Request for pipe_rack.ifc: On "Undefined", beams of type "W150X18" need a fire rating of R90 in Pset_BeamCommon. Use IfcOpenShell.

First a look at what the model holds.

```python
import ifcopenshell
import ifcopenshell.util.element

model = ifcopenshell.open("pipe_rack.ifc")
print(model.schema)
storey = next(s for s in model.by_type("IfcBuildingStorey") if s.Name == "Undefined")
beams = [e for e in ifcopenshell.util.element.get_decomposition(storey) if e.is_a("IfcBeam")]
seen = {}
for e in beams:
    element_type = ifcopenshell.util.element.get_type(e)
    key = (element_type.Name if element_type != e and element_type else None, ifcopenshell.util.element.get_pset(e, "Pset_BeamCommon", "FireRating"))
    seen[key] = seen.get(key, 0) + 1
for (name, value), count in sorted(seen.items(), key=str):
    print(count, "x", name, "|", value)
```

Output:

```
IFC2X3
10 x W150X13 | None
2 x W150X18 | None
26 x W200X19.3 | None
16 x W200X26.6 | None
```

```python
import ifcopenshell
import ifcopenshell.api.pset
import ifcopenshell.util.element

model = ifcopenshell.open("pipe_rack.ifc")

storey = next(s for s in model.by_type("IfcBuildingStorey") if s.Name == "Undefined")
beams = [e for e in ifcopenshell.util.element.get_decomposition(storey) if e.is_a("IfcBeam")]

count = 0
for e in beams:
    element_type = ifcopenshell.util.element.get_type(e)
    if element_type in (None, e) or element_type.Name != "W150X18":
        continue
    found = ifcopenshell.util.element.get_pset(e, "Pset_BeamCommon", should_inherit=False)
    if found:
        pset = model.by_id(found["id"])
        if len(ifcopenshell.util.element.get_elements_by_pset(pset)) > 1:
            pset = ifcopenshell.api.pset.unshare_pset(model, products=[e], pset=pset)[0]
    else:
        pset = ifcopenshell.api.pset.add_pset(model, product=e, name="Pset_BeamCommon")
    ifcopenshell.api.pset.edit_pset(model, pset=pset, properties={"FireRating": "R90"})
    count += 1

print(count, "beams updated")

model.write("pipe_rack_edited.ifc")
```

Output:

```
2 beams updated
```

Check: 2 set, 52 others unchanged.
